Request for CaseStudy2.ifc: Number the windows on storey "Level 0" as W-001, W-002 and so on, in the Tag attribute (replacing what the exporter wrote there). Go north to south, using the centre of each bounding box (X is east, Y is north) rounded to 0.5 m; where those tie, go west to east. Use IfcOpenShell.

First a look at what the model holds.

```python
import ifcopenshell
import ifcopenshell.util.element
import ifcopenshell.util.placement

model = ifcopenshell.open("CaseStudy2.ifc")
print(model.schema)
storey = next(s for s in model.by_type("IfcBuildingStorey") if s.Name == "Level 0")
windows = [e for e in ifcopenshell.util.element.get_decomposition(storey) if e.is_a("IfcWindow")]
for e in sorted(windows, key=lambda e: e.id()):
    origin = ifcopenshell.util.placement.get_local_placement(e.ObjectPlacement)[:3, 3]
    print(e.id(), e.Tag, e.Name, origin.round(2) + 0.0, sep=" | ")
```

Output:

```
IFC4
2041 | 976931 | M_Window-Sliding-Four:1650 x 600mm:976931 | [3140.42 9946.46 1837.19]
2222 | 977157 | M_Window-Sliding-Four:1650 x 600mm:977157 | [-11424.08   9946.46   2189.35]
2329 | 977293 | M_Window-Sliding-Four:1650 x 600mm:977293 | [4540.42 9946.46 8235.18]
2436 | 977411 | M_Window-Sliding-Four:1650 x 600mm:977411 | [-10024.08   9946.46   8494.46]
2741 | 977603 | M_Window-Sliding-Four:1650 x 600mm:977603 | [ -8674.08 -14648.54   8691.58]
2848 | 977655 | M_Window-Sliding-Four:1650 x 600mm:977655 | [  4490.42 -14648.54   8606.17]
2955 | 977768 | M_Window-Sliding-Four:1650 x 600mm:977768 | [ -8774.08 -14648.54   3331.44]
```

```python
import ifcopenshell
import ifcopenshell.geom
import ifcopenshell.util.element
import ifcopenshell.util.shape

model = ifcopenshell.open("CaseStudy2.ifc")
settings = ifcopenshell.geom.settings()
settings.set("use-world-coords", True)


def centre(element):
    shape = ifcopenshell.geom.create_shape(settings, element)
    return ifcopenshell.util.shape.get_bbox_centroid(shape.geometry)


storey = next(s for s in model.by_type("IfcBuildingStorey") if s.Name == "Level 0")
windows = [e for e in ifcopenshell.util.element.get_decomposition(storey) if e.is_a("IfcWindow")]

# Insertion points can sit at a corner or the storey origin, so sort by the geometry (in metres).
centres = {e: centre(e) for e in windows}
windows.sort(key=lambda e: (-round(centres[e][1] / 0.5), centres[e][0]))

for i, e in enumerate(windows, start=1):
    number = f"W-0{i:02d}"
    e.Tag = number
    print(e.id(), number)

model.write("CaseStudy2_v2.ifc")
```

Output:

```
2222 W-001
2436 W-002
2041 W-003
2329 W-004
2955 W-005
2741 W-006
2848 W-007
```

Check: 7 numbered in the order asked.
